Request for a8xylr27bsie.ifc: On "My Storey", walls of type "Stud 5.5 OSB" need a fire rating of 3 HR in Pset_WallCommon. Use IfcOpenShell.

First a look at what the model holds.

```python
import ifcopenshell
import ifcopenshell.util.element

model = ifcopenshell.open("a8xylr27bsie.ifc")
print(model.schema)
storey = next(s for s in model.by_type("IfcBuildingStorey") if s.Name == "My Storey")
walls = [e for e in ifcopenshell.util.element.get_decomposition(storey) if e.is_a("IfcWall")]
seen = {}
for e in walls:
    element_type = ifcopenshell.util.element.get_type(e)
    key = (element_type.Name if element_type != e and element_type else None, ifcopenshell.util.element.get_pset(e, "Pset_WallCommon", "FireRating"))
    seen[key] = seen.get(key, 0) + 1
for (name, value), count in sorted(seen.items(), key=str):
    print(count, "x", name, "|", value)
```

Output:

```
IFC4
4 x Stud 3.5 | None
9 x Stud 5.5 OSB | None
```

```python
import ifcopenshell
import ifcopenshell.api.pset
import ifcopenshell.util.element

model = ifcopenshell.open("a8xylr27bsie.ifc")

storey = next(s for s in model.by_type("IfcBuildingStorey") if s.Name == "My Storey")
walls = [e for e in ifcopenshell.util.element.get_decomposition(storey) if e.is_a("IfcWall")]

count = 0
for e in walls:
    element_type = ifcopenshell.util.element.get_type(e)
    if element_type in (None, e) or element_type.Name != "Stud 5.5 OSB":
        continue
    # add_pset returns the element's existing set when there is one.
    pset = ifcopenshell.api.pset.add_pset(model, product=e, name="Pset_WallCommon")
    ifcopenshell.api.pset.edit_pset(model, pset=pset, properties={"FireRating": "3 HR"})
    count += 1

print(count, "walls updated")

model.write("a8xylr27bsie_v2.ifc")
```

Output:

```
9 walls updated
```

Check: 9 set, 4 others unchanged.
